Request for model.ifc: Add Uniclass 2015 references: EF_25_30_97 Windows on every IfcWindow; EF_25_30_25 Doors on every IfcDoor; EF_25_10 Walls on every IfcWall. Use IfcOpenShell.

First a look at what the model holds.

```python
import ifcopenshell

model = ifcopenshell.open("model.ifc")
print(model.schema)
print("classifications:", [c.Name for c in model.by_type("IfcClassification")])
for ifc_class in ("IfcDoor", "IfcRoof", "IfcStair", "IfcWall", "IfcWindow"):
    print(ifc_class, len(model.by_type(ifc_class)))
```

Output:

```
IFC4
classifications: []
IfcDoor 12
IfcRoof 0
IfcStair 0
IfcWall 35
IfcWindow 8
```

```python
import ifcopenshell
import ifcopenshell.api.classification

model = ifcopenshell.open("model.ifc")

system = ifcopenshell.api.classification.add_classification(model, classification="Uniclass 2015")

codes = {
    "IfcWindow": ("EF_25_30_97", "Windows"),
    "IfcDoor": ("EF_25_30_25", "Doors"),
    "IfcWall": ("EF_25_10", "Walls"),
}
for ifc_class, (code, name) in codes.items():
    products = model.by_type(ifc_class)
    ifcopenshell.api.classification.add_reference(
        model, products=products, classification=system, identification=code, name=name
    )
    print(code, len(products))

model.write("model_edited.ifc")
```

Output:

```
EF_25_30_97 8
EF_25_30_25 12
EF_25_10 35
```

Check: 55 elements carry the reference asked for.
